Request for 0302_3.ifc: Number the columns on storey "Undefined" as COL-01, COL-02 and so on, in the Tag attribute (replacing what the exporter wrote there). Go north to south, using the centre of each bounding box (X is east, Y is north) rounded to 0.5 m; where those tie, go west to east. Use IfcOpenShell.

First a look at what the model holds.

```python
import ifcopenshell
import ifcopenshell.util.element
import ifcopenshell.util.placement

model = ifcopenshell.open("0302_3.ifc")
print(model.schema)
storey = next(s for s in model.by_type("IfcBuildingStorey") if s.Name == "Undefined")
columns = [e for e in ifcopenshell.util.element.get_decomposition(storey) if e.is_a("IfcColumn")]
for e in sorted(columns, key=lambda e: e.id()):
    origin = ifcopenshell.util.placement.get_local_placement(e.ObjectPlacement)[:3, 3]
    print(e.id(), e.Tag, e.Name, origin.round(2) + 0.0, sep=" | ")
```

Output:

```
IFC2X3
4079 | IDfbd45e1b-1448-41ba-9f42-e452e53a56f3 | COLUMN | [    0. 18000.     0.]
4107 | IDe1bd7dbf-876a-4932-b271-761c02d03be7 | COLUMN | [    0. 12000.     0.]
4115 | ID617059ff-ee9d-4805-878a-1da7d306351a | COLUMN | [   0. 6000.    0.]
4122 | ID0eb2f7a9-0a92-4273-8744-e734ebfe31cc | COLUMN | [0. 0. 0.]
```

```python
import ifcopenshell
import ifcopenshell.geom
import ifcopenshell.util.element
import ifcopenshell.util.shape

model = ifcopenshell.open("0302_3.ifc")
settings = ifcopenshell.geom.settings()
settings.set("use-world-coords", True)


def centre(element):
    shape = ifcopenshell.geom.create_shape(settings, element)
    return ifcopenshell.util.shape.get_bbox_centroid(shape.geometry)


storey = next(s for s in model.by_type("IfcBuildingStorey") if s.Name == "Undefined")
columns = [e for e in ifcopenshell.util.element.get_decomposition(storey) if e.is_a("IfcColumn")]

# Insertion points can sit at a corner or the storey origin, so sort by the geometry (in metres).
centres = {e: centre(e) for e in columns}
columns.sort(key=lambda e: (-round(centres[e][1] / 0.5), centres[e][0]))

for i, e in enumerate(columns, start=1):
    number = f"COL-{i:02d}"
    e.Tag = number
    print(e.id(), number)

model.write("0302_3-out.ifc")
```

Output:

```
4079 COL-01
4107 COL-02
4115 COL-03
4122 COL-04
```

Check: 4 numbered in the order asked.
